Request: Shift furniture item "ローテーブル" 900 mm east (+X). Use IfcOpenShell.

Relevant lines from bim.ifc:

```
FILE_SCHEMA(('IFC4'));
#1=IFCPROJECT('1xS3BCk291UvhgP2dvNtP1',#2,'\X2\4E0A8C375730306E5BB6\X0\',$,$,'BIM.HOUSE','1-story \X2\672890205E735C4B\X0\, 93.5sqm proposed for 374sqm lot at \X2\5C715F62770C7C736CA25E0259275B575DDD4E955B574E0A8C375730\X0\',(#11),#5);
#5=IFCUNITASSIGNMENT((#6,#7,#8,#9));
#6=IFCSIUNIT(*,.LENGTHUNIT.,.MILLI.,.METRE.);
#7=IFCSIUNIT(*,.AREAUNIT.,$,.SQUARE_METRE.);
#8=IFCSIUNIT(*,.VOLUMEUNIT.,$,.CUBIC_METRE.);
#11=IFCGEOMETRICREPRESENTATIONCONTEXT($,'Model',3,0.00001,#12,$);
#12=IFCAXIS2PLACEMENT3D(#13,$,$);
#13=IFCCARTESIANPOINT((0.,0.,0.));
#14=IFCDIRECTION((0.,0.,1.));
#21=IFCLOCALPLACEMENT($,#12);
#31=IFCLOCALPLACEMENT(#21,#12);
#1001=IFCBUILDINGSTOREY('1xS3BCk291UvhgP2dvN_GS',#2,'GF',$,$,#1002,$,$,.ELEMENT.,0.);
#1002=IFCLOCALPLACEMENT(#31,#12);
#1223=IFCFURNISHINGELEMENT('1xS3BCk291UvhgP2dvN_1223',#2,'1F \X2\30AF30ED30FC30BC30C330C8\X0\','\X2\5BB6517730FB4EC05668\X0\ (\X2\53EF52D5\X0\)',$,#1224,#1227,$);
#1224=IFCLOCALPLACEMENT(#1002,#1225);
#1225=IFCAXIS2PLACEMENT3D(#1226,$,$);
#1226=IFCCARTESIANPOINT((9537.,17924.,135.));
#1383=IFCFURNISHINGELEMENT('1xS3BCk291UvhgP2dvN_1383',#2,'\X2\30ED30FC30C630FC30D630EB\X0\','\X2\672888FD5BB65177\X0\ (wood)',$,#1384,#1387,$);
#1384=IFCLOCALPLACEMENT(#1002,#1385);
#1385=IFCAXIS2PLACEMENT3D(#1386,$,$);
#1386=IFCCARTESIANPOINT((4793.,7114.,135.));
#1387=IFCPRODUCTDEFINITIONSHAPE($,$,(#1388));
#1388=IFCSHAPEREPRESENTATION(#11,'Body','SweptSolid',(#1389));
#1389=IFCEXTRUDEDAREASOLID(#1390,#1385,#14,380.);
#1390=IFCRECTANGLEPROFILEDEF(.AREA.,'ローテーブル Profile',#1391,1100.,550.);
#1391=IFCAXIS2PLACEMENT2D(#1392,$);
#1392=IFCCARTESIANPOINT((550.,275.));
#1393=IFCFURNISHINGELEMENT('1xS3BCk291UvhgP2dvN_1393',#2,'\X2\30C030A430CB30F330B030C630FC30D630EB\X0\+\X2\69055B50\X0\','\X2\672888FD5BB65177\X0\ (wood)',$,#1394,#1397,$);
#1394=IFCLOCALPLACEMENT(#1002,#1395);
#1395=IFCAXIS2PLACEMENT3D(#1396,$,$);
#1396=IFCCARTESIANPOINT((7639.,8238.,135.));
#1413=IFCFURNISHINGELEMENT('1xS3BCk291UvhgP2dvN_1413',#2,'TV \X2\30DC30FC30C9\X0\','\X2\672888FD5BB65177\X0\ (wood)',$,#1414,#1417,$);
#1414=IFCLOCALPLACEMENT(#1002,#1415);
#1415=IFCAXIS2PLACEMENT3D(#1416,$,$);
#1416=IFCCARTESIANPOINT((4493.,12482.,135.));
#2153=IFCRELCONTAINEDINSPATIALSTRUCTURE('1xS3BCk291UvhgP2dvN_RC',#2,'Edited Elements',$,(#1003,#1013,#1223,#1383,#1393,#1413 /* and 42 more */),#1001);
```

```python
import ifcopenshell
import ifcopenshell.api.geometry
import ifcopenshell.util.placement
import ifcopenshell.util.unit

model = ifcopenshell.open("bim.ifc")
unit_scale = ifcopenshell.util.unit.calculate_unit_scale(model)

item = model.by_id(1383)
matrix = ifcopenshell.util.placement.get_local_placement(item.ObjectPlacement)
matrix[0, 3] += 0.9 / unit_scale
ifcopenshell.api.geometry.edit_object_placement(model, product=item, matrix=matrix, is_si=False)

print(ifcopenshell.util.placement.get_local_placement(item.ObjectPlacement).round(3) + 0.0)

model.write("bim_updated.ifc")
```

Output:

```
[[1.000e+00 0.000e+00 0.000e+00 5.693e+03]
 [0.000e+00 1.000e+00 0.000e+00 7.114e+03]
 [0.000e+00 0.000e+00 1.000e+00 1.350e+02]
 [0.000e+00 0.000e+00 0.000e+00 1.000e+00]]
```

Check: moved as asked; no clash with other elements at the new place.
